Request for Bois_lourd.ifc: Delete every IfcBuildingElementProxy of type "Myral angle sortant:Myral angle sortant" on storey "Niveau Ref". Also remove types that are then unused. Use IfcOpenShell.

First a look at what the model holds.

```python
import ifcopenshell
import ifcopenshell.util.element

model = ifcopenshell.open("Bois_lourd.ifc")
print(model.schema)
storey = next(s for s in model.by_type("IfcBuildingStorey") if s.Name == "Niveau Ref")
proxies = [e for e in ifcopenshell.util.element.get_decomposition(storey) if e.is_a("IfcBuildingElementProxy")]
seen = {}
for e in proxies:
    element_type = ifcopenshell.util.element.get_type(e)
    name = element_type.Name if element_type not in (None, e) else None
    seen[name] = seen.get(name, 0) + 1
for name, count in sorted(seen.items(), key=str):
    print(count, "x", name)
```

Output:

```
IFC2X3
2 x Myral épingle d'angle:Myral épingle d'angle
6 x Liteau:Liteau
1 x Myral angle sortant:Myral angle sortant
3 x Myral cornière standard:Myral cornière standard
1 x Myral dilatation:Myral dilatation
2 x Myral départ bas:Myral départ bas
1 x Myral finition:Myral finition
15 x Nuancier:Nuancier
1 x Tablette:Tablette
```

```python
import ifcopenshell
import ifcopenshell.api.root
import ifcopenshell.util.element

model = ifcopenshell.open("Bois_lourd.ifc")

storey = next(s for s in model.by_type("IfcBuildingStorey") if s.Name == "Niveau Ref")
proxies = [e for e in ifcopenshell.util.element.get_decomposition(storey) if e.is_a("IfcBuildingElementProxy")]
targets = [e for e in proxies if (t := ifcopenshell.util.element.get_type(e)) not in (None, e) and t.Name == "Myral angle sortant:Myral angle sortant"]
types = {ifcopenshell.util.element.get_type(e) for e in targets} - {None, *targets}

for e in targets:
    ifcopenshell.api.root.remove_product(model, product=e)
print(len(targets), "removed")

unused = [t for t in types if not ifcopenshell.util.element.get_types(t)]
for t in unused:
    ifcopenshell.api.root.remove_product(model, product=t)
print(len(unused), "unused types removed")

model.write("Bois_lourd-out.ifc")
```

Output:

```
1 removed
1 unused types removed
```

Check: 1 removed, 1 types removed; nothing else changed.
